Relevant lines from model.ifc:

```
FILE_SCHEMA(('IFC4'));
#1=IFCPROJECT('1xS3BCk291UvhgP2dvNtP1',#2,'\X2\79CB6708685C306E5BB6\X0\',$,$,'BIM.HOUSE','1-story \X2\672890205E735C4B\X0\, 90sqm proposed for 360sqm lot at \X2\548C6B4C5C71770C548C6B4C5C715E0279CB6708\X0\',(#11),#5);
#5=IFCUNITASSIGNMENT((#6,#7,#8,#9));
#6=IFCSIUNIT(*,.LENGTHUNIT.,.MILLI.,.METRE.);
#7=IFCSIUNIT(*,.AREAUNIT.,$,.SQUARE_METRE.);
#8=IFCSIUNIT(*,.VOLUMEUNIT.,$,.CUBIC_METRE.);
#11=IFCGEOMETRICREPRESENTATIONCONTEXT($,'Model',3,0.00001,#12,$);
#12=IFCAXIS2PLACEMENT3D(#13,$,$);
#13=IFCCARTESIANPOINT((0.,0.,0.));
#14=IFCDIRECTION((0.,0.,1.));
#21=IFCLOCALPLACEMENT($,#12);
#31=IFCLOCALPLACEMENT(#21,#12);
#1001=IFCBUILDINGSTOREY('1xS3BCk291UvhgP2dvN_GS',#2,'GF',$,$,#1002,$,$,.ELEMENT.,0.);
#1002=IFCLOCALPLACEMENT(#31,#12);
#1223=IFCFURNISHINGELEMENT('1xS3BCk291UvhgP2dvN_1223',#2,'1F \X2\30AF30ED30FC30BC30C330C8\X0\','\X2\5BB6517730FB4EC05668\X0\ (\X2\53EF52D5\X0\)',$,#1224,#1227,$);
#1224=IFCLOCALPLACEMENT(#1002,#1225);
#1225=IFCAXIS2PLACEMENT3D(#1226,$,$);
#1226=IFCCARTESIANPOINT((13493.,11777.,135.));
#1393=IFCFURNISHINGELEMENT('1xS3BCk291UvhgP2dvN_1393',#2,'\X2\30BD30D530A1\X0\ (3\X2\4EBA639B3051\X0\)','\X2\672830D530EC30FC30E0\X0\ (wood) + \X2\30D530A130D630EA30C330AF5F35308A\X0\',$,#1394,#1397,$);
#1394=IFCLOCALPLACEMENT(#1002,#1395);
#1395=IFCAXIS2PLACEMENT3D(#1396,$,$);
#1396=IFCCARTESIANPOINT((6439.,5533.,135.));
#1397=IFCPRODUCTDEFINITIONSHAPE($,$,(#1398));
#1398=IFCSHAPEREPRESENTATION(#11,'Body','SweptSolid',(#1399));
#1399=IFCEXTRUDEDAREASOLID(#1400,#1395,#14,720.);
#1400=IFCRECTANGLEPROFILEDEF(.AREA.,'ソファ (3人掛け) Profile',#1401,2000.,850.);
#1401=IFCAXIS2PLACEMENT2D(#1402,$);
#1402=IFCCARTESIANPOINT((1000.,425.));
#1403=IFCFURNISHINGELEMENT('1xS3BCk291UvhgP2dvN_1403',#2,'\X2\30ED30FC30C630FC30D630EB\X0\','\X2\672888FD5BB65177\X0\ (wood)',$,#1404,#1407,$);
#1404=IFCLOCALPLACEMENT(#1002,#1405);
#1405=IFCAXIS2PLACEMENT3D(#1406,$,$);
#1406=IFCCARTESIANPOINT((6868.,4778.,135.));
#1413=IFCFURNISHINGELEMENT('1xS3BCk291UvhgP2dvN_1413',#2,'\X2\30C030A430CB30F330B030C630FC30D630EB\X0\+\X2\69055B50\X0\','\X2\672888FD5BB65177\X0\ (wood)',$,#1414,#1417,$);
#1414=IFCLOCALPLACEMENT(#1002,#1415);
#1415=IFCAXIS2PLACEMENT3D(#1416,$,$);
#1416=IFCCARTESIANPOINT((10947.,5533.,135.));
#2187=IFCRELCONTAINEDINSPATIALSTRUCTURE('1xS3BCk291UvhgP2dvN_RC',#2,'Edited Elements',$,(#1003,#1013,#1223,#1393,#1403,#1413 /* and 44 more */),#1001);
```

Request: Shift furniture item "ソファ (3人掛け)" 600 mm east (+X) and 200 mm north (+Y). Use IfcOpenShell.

```python
import ifcopenshell
import ifcopenshell.api.geometry
import ifcopenshell.util.placement

model = ifcopenshell.open("model.ifc")

item = model.by_id(1393)
matrix = ifcopenshell.util.placement.get_local_placement(item.ObjectPlacement)
matrix[0, 3] += 600.0
matrix[1, 3] += 200.0
ifcopenshell.api.geometry.edit_object_placement(model, product=item, matrix=matrix, is_si=False)

print(ifcopenshell.util.placement.get_local_placement(item.ObjectPlacement).round(3) + 0.0)

model.write("model_edited.ifc")
```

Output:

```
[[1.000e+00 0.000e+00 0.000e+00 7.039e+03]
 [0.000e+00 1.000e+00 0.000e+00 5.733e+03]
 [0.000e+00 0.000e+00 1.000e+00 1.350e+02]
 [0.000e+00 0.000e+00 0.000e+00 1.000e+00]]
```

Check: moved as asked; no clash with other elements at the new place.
